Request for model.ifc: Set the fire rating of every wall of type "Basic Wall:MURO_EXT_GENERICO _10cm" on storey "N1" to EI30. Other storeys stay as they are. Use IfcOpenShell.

First a look at what the model holds.

```python
import ifcopenshell
import ifcopenshell.util.element

model = ifcopenshell.open("model.ifc")
print(model.schema)
storey = next(s for s in model.by_type("IfcBuildingStorey") if s.Name == "N1")
walls = [e for e in ifcopenshell.util.element.get_decomposition(storey) if e.is_a("IfcWall")]
seen = {}
for e in walls:
    element_type = ifcopenshell.util.element.get_type(e)
    key = (element_type.Name if element_type != e and element_type else None, ifcopenshell.util.element.get_pset(e, "Pset_WallCommon", "FireRating"))
    seen[key] = seen.get(key, 0) + 1
for (name, value), count in sorted(seen.items(), key=str):
    print(count, "x", name, "|", value)
```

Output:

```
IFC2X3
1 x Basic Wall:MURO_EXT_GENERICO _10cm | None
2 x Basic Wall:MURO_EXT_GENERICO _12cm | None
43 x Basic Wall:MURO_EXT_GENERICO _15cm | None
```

```python
import ifcopenshell
import ifcopenshell.api.pset
import ifcopenshell.util.element

model = ifcopenshell.open("model.ifc")

storey = next(s for s in model.by_type("IfcBuildingStorey") if s.Name == "N1")
walls = [e for e in ifcopenshell.util.element.get_decomposition(storey) if e.is_a("IfcWall")]

count = 0
for e in walls:
    element_type = ifcopenshell.util.element.get_type(e)
    if element_type in (None, e) or element_type.Name != "Basic Wall:MURO_EXT_GENERICO _10cm":
        continue
    # add_pset returns the element's existing set when there is one.
    pset = ifcopenshell.api.pset.add_pset(model, product=e, name="Pset_WallCommon")
    ifcopenshell.api.pset.edit_pset(model, pset=pset, properties={"FireRating": "EI30"})
    count += 1

print(count, "walls updated")

model.write("model_edited.ifc")
```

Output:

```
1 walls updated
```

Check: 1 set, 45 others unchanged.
